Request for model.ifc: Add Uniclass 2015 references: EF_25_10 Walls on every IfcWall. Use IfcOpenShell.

First a look at what the model holds.

```python
import ifcopenshell

model = ifcopenshell.open("model.ifc")
print(model.schema)
print("classifications:", [c.Name for c in model.by_type("IfcClassification")])
for ifc_class in ("IfcDoor", "IfcRoof", "IfcStair", "IfcWall", "IfcWindow"):
    print(ifc_class, len(model.by_type(ifc_class)))
```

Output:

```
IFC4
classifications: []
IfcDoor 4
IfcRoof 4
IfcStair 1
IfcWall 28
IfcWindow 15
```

```python
import ifcopenshell
import ifcopenshell.api.classification

model = ifcopenshell.open("model.ifc")

system = ifcopenshell.api.classification.add_classification(model, classification="Uniclass 2015")

codes = {
    "IfcWall": ("EF_25_10", "Walls"),
}
for ifc_class, (code, name) in codes.items():
    products = model.by_type(ifc_class)
    ifcopenshell.api.classification.add_reference(
        model, products=products, classification=system, identification=code, name=name
    )
    print(code, len(products))

model.write("model_rev.ifc")
```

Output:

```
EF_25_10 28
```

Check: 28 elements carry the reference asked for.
